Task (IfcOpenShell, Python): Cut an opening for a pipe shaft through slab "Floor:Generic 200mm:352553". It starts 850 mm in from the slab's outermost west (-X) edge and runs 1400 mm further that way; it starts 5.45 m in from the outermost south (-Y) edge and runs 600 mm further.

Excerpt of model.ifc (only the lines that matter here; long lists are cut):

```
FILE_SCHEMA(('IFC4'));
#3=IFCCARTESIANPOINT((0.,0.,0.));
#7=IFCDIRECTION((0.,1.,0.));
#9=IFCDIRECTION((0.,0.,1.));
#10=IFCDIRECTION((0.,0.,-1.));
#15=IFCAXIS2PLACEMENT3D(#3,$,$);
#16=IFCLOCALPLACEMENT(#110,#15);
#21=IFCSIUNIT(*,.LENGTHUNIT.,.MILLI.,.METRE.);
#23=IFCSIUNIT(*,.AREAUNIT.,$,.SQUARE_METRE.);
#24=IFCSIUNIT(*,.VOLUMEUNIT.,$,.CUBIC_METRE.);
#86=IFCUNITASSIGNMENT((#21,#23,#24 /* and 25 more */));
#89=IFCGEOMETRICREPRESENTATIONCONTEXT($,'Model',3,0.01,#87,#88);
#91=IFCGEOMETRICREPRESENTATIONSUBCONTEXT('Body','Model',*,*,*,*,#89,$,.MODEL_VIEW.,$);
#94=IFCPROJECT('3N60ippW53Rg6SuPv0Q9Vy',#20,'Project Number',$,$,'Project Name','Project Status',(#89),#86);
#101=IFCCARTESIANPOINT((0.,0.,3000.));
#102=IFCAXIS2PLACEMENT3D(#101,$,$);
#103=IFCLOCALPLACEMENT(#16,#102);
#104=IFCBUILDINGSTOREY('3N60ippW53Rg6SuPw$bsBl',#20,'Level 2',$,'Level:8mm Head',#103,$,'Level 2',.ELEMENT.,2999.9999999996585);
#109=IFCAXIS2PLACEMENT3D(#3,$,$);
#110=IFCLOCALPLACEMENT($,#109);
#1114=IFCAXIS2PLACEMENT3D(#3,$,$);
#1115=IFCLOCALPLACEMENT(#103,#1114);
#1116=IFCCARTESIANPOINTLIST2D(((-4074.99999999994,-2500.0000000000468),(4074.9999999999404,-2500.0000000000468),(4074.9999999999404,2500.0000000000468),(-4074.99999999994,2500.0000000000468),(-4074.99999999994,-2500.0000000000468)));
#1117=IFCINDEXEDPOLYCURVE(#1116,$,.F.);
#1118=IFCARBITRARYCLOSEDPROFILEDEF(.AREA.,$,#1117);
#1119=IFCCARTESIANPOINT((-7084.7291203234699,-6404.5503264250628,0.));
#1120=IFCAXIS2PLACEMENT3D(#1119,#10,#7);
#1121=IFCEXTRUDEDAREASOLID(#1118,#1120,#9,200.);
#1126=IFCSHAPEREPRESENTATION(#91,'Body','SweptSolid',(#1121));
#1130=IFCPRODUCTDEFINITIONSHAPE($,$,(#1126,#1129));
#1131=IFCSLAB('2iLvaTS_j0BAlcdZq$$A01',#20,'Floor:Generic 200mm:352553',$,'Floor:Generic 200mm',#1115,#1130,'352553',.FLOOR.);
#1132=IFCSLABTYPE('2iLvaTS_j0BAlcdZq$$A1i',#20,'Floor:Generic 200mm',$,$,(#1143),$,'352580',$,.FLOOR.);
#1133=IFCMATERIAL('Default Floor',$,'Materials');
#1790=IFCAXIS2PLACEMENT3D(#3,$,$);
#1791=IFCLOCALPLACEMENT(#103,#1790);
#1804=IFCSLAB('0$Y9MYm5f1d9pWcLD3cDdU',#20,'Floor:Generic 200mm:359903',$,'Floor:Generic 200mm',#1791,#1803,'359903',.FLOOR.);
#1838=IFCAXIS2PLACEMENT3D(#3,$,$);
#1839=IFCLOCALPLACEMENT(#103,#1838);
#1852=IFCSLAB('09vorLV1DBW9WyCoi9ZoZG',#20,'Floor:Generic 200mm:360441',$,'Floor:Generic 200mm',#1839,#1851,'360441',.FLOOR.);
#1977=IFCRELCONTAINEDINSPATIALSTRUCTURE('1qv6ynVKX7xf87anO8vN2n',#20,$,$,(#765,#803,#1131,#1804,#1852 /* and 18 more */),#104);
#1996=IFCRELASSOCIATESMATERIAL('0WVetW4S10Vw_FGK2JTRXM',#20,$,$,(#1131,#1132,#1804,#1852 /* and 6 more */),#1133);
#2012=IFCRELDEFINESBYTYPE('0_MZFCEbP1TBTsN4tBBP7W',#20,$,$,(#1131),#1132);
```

```python
import numpy as np
import ifcopenshell
import ifcopenshell.api.feature
import ifcopenshell.api.geometry
import ifcopenshell.api.root
import ifcopenshell.geom
import ifcopenshell.util.placement
import ifcopenshell.util.representation
import ifcopenshell.util.shape
import ifcopenshell.util.unit

model = ifcopenshell.open("model.ifc")
unit_scale = ifcopenshell.util.unit.calculate_unit_scale(model)
settings = ifcopenshell.geom.settings()


def volume(element):
    """Net volume in cubic metres, openings subtracted."""
    shape = ifcopenshell.geom.create_shape(settings, element)
    return ifcopenshell.util.shape.get_volume(shape.geometry)


slab = model.by_guid("2iLvaTS_j0BAlcdZq$$A01")
before = volume(slab)

# Extent in the slab's own axes, in metres. The edges named are its -X and -Y sides.
slab_shape = ifcopenshell.geom.create_shape(settings, slab)
vertices = ifcopenshell.util.shape.get_vertices(slab_shape.geometry)
x_min, y_min, bottom = vertices.min(axis=0)
top = vertices[:, 2].max()

opening = ifcopenshell.api.root.create_entity(model, ifc_class="IfcOpeningElement", name="Pipe shaft opening", predefined_type="OPENING")
context = ifcopenshell.util.representation.get_context(model, "Model", "Body", "MODEL_VIEW")
width, depth = 1.4, 0.6
outline = [(0.0, 0.0), (width, 0.0), (width, depth), (0.0, depth), (0.0, 0.0)]
# Overshoot both faces by 50 mm so the cut is clean.
shape = ifcopenshell.api.geometry.add_slab_representation(
    model, context=context, depth=top - bottom + 0.1, polyline=outline
)
ifcopenshell.api.geometry.assign_representation(model, product=opening, representation=shape)

matrix = ifcopenshell.util.placement.get_local_placement(slab.ObjectPlacement)
matrix[:, 3] = matrix @ np.append(np.array([x_min + 0.85, y_min + 5.45, bottom - 0.05]) / unit_scale, 1.0)
ifcopenshell.api.geometry.edit_object_placement(model, product=opening, matrix=matrix, is_si=False)
ifcopenshell.api.feature.add_feature(model, feature=opening, element=slab)

after = volume(slab)

print(f"slab volume {before:.3f} -> {after:.3f} m3")

model.write("model_updated.ifc")
```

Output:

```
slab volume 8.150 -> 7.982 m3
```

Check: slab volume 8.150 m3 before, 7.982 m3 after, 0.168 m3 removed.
